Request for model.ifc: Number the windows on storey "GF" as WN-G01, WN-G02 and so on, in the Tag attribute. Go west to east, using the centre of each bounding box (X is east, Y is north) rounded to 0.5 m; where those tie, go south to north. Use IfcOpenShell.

First a look at what the model holds.

```python
import ifcopenshell
import ifcopenshell.util.element
import ifcopenshell.util.placement

model = ifcopenshell.open("model.ifc")
print(model.schema)
storey = next(s for s in model.by_type("IfcBuildingStorey") if s.Name == "GF")
windows = [e for e in ifcopenshell.util.element.get_decomposition(storey) if e.is_a("IfcWindow")]
for e in sorted(windows, key=lambda e: e.id()):
    origin = ifcopenshell.util.placement.get_local_placement(e.ObjectPlacement)[:3, 3]
    print(e.id(), e.Tag, e.Name, origin.round(2) + 0.0, sep=" | ")
```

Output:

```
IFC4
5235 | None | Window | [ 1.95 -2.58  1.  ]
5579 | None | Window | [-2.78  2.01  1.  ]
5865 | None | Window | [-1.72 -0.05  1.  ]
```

```python
import ifcopenshell
import ifcopenshell.geom
import ifcopenshell.util.element
import ifcopenshell.util.shape

model = ifcopenshell.open("model.ifc")
settings = ifcopenshell.geom.settings()
settings.set("use-world-coords", True)


def centre(element):
    shape = ifcopenshell.geom.create_shape(settings, element)
    return ifcopenshell.util.shape.get_bbox_centroid(shape.geometry)


storey = next(s for s in model.by_type("IfcBuildingStorey") if s.Name == "GF")
windows = [e for e in ifcopenshell.util.element.get_decomposition(storey) if e.is_a("IfcWindow")]

# Insertion points can sit at a corner or the storey origin, so sort by the geometry (in metres).
centres = {e: centre(e) for e in windows}
windows.sort(key=lambda e: (round(centres[e][0] / 0.5), centres[e][1]))

for i, e in enumerate(windows, start=1):
    number = f"WN-G{i:02d}"
    e.Tag = number
    print(e.id(), number)

model.write("model_updated.ifc")
```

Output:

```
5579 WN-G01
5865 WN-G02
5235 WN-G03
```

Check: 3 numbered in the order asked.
